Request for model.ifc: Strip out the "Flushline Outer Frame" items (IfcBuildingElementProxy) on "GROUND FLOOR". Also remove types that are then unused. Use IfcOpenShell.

First a look at what the model holds.

```python
import ifcopenshell
import ifcopenshell.util.element

model = ifcopenshell.open("model.ifc")
print(model.schema)
storey = next(s for s in model.by_type("IfcBuildingStorey") if s.Name == "GROUND FLOOR")
proxies = [e for e in ifcopenshell.util.element.get_decomposition(storey) if e.is_a("IfcBuildingElementProxy")]
seen = {}
for e in proxies:
    element_type = ifcopenshell.util.element.get_type(e)
    name = element_type.Name if element_type not in (None, e) else None
    seen[name] = seen.get(name, 0) + 1
for name, count in sorted(seen.items(), key=str):
    print(count, "x", name)
```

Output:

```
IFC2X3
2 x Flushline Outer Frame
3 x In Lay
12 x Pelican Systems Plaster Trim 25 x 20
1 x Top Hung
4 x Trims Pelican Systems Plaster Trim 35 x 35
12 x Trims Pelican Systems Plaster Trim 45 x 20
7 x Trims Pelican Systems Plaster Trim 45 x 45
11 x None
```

```python
import ifcopenshell
import ifcopenshell.api.root
import ifcopenshell.util.element

model = ifcopenshell.open("model.ifc")

storey = next(s for s in model.by_type("IfcBuildingStorey") if s.Name == "GROUND FLOOR")
proxies = [e for e in ifcopenshell.util.element.get_decomposition(storey) if e.is_a("IfcBuildingElementProxy")]
targets = [e for e in proxies if (t := ifcopenshell.util.element.get_type(e)) not in (None, e) and t.Name == "Flushline Outer Frame"]
types = {ifcopenshell.util.element.get_type(e) for e in targets} - {None, *targets}

for e in targets:
    ifcopenshell.api.root.remove_product(model, product=e)
print(len(targets), "removed")

unused = [t for t in types if not ifcopenshell.util.element.get_types(t)]
for t in unused:
    ifcopenshell.api.root.remove_product(model, product=t)
print(len(unused), "unused types removed")

model.write("model_edited.ifc")
```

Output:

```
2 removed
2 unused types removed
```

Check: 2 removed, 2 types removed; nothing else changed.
